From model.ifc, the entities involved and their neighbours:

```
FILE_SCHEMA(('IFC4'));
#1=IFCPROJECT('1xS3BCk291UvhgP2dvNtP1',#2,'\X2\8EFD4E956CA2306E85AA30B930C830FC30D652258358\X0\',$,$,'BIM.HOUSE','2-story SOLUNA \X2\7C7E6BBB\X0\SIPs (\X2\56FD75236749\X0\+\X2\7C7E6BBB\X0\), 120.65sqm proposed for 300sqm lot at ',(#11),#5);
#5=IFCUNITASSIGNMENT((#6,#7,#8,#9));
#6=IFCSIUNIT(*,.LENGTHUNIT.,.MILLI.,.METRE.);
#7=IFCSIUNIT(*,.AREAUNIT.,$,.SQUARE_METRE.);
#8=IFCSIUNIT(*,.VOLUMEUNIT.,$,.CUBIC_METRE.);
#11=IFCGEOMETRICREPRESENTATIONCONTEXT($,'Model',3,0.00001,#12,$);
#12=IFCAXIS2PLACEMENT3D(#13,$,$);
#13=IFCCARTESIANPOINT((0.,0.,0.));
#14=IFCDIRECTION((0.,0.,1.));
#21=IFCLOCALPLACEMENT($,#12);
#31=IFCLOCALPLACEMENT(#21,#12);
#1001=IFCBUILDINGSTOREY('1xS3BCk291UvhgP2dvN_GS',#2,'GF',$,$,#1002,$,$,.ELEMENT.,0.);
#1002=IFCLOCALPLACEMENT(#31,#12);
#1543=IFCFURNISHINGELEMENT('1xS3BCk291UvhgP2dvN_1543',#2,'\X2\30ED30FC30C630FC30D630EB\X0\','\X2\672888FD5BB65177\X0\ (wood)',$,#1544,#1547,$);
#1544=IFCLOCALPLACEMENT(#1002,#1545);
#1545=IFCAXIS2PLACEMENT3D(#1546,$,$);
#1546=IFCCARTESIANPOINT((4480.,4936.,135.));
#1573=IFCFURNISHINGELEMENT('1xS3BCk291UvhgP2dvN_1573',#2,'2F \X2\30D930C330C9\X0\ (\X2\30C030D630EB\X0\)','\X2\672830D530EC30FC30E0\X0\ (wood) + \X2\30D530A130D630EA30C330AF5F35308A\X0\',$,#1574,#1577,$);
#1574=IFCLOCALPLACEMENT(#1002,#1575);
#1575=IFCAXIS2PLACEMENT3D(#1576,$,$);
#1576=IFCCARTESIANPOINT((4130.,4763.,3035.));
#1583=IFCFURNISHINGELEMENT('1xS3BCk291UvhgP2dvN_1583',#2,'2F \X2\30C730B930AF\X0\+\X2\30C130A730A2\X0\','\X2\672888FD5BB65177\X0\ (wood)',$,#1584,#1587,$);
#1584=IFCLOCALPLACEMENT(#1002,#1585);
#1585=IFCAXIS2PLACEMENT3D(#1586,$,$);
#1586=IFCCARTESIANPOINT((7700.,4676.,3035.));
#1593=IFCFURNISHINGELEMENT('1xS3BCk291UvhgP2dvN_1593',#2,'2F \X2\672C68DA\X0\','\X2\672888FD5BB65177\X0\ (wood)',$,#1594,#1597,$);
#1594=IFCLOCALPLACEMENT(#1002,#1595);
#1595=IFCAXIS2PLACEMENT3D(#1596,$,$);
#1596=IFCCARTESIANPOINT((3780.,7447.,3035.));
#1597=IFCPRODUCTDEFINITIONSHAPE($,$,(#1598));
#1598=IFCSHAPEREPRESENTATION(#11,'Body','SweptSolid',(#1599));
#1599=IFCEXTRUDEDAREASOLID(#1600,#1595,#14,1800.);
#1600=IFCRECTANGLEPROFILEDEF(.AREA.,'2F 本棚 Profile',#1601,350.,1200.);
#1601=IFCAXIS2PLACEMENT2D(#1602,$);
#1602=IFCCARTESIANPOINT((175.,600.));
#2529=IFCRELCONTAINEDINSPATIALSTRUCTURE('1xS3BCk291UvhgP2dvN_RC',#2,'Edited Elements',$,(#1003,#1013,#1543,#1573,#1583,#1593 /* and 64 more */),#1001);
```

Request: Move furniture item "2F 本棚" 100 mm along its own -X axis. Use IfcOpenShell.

```python
import ifcopenshell
import ifcopenshell.api.geometry
import ifcopenshell.util.placement

model = ifcopenshell.open("model.ifc")

item = model.by_guid("1xS3BCk291UvhgP2dvN_1593")
matrix = ifcopenshell.util.placement.get_local_placement(item.ObjectPlacement)
matrix[:3, 3] -= matrix[:3, 0] * 100.0
ifcopenshell.api.geometry.edit_object_placement(model, product=item, matrix=matrix, is_si=False)

print(ifcopenshell.util.placement.get_local_placement(item.ObjectPlacement).round(3) + 0.0)

model.write("model_v2.ifc")
```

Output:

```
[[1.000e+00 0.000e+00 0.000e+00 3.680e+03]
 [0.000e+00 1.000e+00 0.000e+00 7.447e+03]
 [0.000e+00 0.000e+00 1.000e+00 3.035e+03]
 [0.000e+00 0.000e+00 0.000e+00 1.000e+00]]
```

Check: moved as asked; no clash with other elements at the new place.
